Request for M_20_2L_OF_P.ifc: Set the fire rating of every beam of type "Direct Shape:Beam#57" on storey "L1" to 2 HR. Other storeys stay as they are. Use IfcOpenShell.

First a look at what the model holds.

```python
import ifcopenshell
import ifcopenshell.util.element

model = ifcopenshell.open("M_20_2L_OF_P.ifc")
print(model.schema)
storey = next(s for s in model.by_type("IfcBuildingStorey") if s.Name == "L1")
beams = [e for e in ifcopenshell.util.element.get_decomposition(storey) if e.is_a("IfcBeam")]
seen = {}
for e in beams:
    element_type = ifcopenshell.util.element.get_type(e)
    key = (element_type.Name if element_type != e and element_type else None, ifcopenshell.util.element.get_pset(e, "Pset_BeamCommon", "FireRating"))
    seen[key] = seen.get(key, 0) + 1
for (name, value), count in sorted(seen.items(), key=str):
    print(count, "x", name, "|", value)
```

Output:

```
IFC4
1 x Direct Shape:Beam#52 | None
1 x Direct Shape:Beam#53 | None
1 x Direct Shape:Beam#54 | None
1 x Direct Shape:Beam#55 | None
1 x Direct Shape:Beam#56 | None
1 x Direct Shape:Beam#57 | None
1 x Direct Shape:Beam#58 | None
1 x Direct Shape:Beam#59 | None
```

```python
import ifcopenshell
import ifcopenshell.api.pset
import ifcopenshell.util.element

model = ifcopenshell.open("M_20_2L_OF_P.ifc")

storey = next(s for s in model.by_type("IfcBuildingStorey") if s.Name == "L1")
beams = [e for e in ifcopenshell.util.element.get_decomposition(storey) if e.is_a("IfcBeam")]

count = 0
for e in beams:
    element_type = ifcopenshell.util.element.get_type(e)
    if element_type in (None, e) or element_type.Name != "Direct Shape:Beam#57":
        continue
    # add_pset returns the element's existing set when there is one.
    pset = ifcopenshell.api.pset.add_pset(model, product=e, name="Pset_BeamCommon")
    ifcopenshell.api.pset.edit_pset(model, pset=pset, properties={"FireRating": "2 HR"})
    count += 1

print(count, "beams updated")

model.write("M_20_2L_OF_P-out.ifc")
```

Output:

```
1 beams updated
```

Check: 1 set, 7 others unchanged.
